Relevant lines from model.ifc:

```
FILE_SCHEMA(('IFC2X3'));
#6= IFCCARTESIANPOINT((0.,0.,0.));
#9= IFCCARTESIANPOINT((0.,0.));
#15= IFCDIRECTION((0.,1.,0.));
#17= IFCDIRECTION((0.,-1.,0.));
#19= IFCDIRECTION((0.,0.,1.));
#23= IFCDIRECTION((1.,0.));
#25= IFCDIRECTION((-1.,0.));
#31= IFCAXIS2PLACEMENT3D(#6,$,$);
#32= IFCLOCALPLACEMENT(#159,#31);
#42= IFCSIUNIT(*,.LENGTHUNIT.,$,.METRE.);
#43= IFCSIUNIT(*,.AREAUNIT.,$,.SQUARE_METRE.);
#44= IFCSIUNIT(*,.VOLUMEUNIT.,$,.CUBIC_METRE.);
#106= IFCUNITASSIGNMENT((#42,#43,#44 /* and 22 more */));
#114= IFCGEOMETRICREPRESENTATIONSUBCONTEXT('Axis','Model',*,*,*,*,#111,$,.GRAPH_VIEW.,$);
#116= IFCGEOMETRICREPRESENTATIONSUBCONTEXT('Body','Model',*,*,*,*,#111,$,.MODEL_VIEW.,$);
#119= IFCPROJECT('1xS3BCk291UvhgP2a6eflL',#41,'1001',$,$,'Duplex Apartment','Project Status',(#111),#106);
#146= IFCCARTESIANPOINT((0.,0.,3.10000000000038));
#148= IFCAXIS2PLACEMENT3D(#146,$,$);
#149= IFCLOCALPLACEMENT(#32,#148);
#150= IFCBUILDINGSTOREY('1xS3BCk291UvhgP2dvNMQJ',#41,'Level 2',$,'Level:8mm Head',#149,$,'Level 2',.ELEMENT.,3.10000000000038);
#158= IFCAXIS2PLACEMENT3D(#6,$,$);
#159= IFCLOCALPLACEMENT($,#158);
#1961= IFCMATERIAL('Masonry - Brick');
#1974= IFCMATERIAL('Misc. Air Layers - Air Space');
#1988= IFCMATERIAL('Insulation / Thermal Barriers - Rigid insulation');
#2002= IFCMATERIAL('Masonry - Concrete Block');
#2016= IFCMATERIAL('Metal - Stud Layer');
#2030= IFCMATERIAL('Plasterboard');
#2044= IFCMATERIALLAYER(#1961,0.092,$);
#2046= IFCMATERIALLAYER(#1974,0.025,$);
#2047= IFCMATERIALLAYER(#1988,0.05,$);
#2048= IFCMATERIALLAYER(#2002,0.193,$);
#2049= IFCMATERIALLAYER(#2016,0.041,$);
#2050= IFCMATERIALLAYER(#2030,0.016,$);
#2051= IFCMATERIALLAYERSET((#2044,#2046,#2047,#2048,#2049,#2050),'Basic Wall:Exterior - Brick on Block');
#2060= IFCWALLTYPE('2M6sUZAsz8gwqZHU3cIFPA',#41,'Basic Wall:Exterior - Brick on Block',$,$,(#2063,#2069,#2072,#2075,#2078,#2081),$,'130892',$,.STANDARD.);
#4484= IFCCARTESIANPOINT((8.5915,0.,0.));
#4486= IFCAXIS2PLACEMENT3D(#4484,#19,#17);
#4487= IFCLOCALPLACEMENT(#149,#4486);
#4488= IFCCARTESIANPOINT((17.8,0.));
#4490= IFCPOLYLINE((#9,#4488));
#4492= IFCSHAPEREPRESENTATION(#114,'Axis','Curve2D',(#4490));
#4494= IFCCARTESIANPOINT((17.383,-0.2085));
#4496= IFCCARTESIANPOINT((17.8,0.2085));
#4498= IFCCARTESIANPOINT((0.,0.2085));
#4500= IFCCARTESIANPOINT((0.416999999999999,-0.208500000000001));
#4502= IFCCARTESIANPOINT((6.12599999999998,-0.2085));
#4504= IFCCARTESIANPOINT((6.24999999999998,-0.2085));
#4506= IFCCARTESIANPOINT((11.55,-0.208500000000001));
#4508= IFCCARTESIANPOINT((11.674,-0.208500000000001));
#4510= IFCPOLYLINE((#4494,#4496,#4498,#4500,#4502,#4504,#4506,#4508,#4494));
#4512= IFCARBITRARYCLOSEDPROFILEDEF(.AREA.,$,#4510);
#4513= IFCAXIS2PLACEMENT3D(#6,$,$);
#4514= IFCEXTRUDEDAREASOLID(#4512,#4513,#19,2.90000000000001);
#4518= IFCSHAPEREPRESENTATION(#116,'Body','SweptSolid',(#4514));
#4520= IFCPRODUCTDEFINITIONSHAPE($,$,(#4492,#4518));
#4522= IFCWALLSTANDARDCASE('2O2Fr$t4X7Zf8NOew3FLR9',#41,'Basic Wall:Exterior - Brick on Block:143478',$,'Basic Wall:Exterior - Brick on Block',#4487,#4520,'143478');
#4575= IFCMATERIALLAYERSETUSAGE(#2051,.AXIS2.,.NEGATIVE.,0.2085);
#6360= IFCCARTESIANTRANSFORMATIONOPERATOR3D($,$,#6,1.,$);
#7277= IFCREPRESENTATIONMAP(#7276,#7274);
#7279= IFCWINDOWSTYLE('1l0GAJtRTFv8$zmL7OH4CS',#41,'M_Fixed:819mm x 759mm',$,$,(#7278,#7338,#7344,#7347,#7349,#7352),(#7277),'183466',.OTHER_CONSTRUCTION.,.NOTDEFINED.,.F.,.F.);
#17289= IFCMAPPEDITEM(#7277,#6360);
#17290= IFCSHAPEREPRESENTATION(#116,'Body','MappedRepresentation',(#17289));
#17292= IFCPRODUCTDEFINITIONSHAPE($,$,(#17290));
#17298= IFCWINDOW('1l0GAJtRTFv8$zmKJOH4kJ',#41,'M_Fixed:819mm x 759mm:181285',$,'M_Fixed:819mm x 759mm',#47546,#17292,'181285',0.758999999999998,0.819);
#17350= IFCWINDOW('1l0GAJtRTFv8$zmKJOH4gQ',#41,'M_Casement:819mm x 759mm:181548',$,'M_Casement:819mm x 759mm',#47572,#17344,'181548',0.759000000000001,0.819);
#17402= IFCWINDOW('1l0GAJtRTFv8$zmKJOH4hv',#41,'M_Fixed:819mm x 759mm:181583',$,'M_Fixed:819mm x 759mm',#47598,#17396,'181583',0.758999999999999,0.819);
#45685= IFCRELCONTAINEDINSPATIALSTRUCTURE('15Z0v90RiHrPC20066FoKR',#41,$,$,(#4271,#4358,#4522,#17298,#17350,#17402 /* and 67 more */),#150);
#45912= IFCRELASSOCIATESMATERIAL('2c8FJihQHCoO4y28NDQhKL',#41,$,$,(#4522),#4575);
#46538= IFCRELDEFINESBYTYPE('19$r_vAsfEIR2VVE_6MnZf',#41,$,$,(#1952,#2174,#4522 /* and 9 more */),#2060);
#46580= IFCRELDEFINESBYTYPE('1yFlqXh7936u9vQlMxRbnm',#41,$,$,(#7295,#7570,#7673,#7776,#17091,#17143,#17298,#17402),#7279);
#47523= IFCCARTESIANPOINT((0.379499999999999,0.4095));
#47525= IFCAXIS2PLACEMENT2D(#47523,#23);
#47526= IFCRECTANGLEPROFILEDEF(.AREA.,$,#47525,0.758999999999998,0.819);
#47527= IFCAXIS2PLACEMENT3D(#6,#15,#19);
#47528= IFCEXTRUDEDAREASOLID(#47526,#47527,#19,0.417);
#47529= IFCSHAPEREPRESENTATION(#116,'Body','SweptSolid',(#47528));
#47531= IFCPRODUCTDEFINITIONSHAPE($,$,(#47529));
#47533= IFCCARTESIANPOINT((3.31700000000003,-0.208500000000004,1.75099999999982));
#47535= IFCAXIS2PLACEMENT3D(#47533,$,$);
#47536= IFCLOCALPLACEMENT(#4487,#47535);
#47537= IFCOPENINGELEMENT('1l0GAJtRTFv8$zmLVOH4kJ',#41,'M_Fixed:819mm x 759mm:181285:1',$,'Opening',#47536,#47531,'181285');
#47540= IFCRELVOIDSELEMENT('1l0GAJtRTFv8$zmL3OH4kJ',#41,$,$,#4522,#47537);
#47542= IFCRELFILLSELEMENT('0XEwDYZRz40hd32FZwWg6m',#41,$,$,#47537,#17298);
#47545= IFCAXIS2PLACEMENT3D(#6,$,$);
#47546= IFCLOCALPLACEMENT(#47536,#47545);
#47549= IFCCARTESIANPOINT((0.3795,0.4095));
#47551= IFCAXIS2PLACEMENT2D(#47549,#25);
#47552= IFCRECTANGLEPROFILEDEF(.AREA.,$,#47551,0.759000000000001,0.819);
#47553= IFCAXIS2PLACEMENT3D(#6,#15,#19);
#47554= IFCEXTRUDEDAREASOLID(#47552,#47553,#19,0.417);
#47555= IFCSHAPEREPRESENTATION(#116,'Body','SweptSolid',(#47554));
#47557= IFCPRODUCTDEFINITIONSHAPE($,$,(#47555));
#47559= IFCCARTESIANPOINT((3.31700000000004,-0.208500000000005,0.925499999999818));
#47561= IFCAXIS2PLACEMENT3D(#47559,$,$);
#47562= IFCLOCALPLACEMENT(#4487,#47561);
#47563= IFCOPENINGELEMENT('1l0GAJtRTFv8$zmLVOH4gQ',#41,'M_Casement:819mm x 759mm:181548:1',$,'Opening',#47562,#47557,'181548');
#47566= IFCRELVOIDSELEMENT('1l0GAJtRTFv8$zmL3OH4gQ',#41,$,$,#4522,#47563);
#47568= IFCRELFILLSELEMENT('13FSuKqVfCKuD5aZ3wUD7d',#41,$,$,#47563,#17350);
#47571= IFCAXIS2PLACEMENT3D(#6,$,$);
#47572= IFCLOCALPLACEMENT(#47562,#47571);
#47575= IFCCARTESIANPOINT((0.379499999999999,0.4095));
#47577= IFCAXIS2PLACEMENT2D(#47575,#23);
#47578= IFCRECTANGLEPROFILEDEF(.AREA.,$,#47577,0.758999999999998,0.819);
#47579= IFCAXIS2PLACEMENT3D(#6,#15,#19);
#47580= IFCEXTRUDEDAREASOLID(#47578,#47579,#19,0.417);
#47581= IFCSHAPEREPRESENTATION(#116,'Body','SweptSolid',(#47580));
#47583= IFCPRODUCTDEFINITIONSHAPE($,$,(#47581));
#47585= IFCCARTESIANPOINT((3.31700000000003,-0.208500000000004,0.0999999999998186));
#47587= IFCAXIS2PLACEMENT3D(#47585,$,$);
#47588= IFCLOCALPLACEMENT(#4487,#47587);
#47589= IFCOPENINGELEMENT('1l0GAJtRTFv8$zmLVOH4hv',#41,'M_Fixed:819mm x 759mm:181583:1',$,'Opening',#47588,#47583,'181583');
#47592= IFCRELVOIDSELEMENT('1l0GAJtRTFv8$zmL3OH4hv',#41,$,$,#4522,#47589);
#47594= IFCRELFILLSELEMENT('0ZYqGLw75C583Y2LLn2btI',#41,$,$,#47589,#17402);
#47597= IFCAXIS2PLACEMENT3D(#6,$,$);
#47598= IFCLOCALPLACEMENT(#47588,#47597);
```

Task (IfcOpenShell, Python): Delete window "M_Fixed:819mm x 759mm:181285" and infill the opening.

```python
import ifcopenshell
import ifcopenshell.api.feature
import ifcopenshell.api.root
import ifcopenshell.geom
import ifcopenshell.util.shape

model = ifcopenshell.open("model.ifc")
settings = ifcopenshell.geom.settings()


def volume(element):
    """Net volume in cubic metres, openings subtracted."""
    shape = ifcopenshell.geom.create_shape(settings, element)
    return ifcopenshell.util.shape.get_volume(shape.geometry)


window = model.by_guid("1l0GAJtRTFv8$zmKJOH4kJ")
opening = window.FillsVoids[0].RelatingOpeningElement
wall = opening.VoidsElements[0].RelatingBuildingElement
before = volume(wall)

ifcopenshell.api.root.remove_product(model, product=window)
ifcopenshell.api.feature.remove_feature(model, feature=opening)

after = volume(wall)

print(f"wall volume {before:.3f} -> {after:.3f} m3")

model.write("model_edited.ifc")
```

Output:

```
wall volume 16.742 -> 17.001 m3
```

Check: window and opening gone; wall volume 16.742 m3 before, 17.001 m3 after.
